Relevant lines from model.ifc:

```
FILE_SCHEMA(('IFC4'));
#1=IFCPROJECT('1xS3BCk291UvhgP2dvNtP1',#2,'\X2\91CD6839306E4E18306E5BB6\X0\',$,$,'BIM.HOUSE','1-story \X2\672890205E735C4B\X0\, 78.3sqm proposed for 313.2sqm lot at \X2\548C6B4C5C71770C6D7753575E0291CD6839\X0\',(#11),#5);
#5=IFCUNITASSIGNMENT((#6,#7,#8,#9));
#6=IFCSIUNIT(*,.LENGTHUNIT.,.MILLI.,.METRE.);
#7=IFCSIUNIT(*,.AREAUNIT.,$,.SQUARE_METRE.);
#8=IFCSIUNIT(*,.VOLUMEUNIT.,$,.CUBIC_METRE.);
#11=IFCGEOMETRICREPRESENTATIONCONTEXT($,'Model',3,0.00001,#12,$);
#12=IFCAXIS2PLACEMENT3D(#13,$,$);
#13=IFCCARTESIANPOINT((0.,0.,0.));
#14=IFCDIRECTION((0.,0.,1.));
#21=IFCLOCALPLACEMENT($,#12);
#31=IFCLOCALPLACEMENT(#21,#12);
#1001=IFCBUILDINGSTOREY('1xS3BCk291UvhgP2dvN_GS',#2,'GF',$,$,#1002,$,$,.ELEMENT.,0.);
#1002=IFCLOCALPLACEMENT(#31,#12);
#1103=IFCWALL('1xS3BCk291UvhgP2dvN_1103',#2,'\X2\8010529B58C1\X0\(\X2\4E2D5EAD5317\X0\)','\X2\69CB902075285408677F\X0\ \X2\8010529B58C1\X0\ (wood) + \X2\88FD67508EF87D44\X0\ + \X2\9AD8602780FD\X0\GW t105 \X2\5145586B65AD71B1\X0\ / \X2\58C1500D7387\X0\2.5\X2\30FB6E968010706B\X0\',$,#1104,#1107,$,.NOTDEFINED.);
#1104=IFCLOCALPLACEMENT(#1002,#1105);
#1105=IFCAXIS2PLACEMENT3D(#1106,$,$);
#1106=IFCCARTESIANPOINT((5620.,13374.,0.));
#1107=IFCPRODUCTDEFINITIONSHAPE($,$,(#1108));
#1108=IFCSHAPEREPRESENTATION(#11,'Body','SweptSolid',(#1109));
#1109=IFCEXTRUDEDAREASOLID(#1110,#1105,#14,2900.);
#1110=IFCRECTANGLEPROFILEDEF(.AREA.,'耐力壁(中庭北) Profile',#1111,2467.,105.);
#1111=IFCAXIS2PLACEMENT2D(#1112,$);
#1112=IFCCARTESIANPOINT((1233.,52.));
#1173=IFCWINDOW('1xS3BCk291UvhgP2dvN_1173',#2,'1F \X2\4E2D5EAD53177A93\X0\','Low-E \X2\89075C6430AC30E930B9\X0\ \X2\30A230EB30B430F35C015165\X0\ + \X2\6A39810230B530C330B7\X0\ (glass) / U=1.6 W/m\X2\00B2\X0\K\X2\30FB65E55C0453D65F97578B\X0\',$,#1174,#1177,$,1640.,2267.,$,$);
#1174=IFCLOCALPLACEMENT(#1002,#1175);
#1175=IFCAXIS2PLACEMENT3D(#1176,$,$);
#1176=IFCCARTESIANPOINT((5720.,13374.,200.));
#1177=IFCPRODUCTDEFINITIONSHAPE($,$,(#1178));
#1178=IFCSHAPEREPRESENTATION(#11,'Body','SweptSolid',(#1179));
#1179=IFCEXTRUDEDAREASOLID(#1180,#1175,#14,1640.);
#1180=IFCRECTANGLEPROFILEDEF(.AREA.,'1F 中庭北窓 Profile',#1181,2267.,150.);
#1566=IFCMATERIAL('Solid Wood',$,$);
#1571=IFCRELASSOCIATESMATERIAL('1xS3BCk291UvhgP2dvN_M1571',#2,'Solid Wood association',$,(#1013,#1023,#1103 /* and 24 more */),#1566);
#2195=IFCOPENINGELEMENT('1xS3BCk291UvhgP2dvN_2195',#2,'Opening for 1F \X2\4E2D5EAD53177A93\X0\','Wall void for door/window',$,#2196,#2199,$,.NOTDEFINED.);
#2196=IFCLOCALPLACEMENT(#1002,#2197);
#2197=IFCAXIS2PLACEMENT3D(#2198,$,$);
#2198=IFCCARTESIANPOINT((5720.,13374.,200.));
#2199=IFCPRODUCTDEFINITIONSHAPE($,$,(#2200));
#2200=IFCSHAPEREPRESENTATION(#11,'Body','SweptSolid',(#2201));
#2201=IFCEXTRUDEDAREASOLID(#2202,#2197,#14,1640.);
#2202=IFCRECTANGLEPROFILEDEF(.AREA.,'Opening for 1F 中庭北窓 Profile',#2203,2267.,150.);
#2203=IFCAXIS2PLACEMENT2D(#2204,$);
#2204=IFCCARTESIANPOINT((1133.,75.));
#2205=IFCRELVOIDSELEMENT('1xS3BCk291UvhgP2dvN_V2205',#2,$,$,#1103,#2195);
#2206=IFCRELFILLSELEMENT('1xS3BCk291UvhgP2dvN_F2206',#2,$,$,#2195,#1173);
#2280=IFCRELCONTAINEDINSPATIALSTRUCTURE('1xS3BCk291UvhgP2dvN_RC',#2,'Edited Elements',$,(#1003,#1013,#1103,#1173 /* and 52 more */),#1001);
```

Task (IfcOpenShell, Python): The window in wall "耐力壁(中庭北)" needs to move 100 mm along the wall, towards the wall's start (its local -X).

```python
import ifcopenshell
import ifcopenshell.api.geometry
import ifcopenshell.util.placement

model = ifcopenshell.open("model.ifc")

window = model.by_id(1173)
opening = window.FillsVoids[0].RelatingOpeningElement
wall = opening.VoidsElements[0].RelatingBuildingElement

wall_matrix = ifcopenshell.util.placement.get_local_placement(wall.ObjectPlacement)
shift = wall_matrix[:3, 0] * -100.0
before = ifcopenshell.util.placement.get_local_placement(window.ObjectPlacement)[:3, 3].copy()

# The window is not placed relative to its opening, so move both.
for product in (opening, window):
    matrix = ifcopenshell.util.placement.get_local_placement(product.ObjectPlacement)
    matrix[:3, 3] += shift
    ifcopenshell.api.geometry.edit_object_placement(model, product=product, matrix=matrix, is_si=False)

after = ifcopenshell.util.placement.get_local_placement(window.ObjectPlacement)[:3, 3]
print("window moved by", (after - before).round(3) + 0.0)

model.write("model-out.ifc")
```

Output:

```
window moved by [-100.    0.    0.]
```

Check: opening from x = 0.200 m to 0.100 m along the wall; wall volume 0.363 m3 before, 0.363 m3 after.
